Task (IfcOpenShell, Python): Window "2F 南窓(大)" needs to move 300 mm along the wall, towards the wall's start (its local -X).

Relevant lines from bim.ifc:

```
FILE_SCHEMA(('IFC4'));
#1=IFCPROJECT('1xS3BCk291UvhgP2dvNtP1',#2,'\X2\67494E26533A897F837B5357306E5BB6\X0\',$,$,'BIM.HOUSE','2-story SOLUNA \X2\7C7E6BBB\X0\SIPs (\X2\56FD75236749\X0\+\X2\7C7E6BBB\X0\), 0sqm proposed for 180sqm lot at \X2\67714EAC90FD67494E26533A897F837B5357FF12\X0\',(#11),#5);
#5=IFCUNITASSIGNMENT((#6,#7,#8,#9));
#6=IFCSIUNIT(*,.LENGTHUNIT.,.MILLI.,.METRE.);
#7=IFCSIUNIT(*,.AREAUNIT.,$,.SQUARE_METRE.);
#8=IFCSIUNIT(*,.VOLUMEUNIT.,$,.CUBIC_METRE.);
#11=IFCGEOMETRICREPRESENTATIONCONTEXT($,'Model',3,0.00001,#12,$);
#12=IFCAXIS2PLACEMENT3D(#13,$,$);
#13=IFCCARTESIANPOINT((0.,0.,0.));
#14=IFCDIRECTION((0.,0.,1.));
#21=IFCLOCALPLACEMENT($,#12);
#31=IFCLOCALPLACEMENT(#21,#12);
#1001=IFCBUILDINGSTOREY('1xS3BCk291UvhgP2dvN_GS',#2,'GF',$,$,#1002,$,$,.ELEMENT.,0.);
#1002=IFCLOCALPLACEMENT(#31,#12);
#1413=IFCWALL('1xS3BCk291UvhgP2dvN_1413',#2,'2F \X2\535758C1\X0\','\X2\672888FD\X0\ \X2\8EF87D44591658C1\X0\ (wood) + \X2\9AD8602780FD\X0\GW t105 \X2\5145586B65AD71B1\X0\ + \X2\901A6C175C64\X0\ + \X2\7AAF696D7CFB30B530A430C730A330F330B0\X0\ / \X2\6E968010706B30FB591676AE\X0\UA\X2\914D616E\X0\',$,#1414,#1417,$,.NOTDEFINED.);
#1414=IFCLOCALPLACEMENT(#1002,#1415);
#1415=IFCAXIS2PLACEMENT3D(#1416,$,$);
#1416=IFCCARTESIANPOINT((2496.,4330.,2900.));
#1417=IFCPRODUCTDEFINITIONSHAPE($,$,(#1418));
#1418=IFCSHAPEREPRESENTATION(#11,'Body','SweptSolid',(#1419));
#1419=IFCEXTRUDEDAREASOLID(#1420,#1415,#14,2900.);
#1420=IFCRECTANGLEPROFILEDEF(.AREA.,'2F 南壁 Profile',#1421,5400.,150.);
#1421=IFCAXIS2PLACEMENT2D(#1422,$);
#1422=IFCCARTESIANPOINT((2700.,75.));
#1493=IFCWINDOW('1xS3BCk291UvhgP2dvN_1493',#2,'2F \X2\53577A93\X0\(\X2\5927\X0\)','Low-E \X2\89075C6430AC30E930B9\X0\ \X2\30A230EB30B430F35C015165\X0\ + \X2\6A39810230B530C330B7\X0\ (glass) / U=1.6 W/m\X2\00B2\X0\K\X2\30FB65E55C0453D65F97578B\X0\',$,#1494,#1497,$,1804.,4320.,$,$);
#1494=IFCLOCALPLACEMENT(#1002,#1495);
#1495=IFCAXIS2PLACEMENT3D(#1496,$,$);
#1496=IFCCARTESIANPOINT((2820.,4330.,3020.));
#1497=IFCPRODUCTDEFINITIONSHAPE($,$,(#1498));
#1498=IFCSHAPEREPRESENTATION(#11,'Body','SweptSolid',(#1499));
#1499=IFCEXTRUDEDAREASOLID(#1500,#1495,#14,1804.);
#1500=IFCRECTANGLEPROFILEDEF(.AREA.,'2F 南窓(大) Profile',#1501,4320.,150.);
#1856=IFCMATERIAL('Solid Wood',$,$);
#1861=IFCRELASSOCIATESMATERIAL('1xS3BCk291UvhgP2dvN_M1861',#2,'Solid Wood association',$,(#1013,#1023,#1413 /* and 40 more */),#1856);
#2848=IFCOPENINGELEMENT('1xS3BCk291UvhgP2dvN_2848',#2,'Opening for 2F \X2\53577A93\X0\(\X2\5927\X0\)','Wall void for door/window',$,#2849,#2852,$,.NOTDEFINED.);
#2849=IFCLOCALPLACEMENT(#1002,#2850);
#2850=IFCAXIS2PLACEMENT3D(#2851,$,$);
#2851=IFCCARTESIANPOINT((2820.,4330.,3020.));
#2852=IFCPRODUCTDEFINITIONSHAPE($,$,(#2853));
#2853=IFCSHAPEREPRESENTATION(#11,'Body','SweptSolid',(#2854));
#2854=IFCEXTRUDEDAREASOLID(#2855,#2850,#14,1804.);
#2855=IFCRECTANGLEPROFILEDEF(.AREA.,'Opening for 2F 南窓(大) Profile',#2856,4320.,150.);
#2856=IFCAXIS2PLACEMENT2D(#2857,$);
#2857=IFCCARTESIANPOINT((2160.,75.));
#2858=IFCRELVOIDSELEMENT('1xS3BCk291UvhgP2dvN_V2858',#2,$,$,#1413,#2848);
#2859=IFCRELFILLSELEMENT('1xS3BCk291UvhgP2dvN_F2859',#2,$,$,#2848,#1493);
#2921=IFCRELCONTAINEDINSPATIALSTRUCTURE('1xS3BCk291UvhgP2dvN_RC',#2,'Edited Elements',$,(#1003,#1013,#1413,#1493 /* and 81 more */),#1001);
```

```python
import ifcopenshell
import ifcopenshell.api.geometry
import ifcopenshell.util.placement

model = ifcopenshell.open("bim.ifc")

window = model.by_guid("1xS3BCk291UvhgP2dvN_1493")
opening = window.FillsVoids[0].RelatingOpeningElement
wall = opening.VoidsElements[0].RelatingBuildingElement

wall_matrix = ifcopenshell.util.placement.get_local_placement(wall.ObjectPlacement)
shift = wall_matrix[:3, 0] * -300.0
before = ifcopenshell.util.placement.get_local_placement(window.ObjectPlacement)[:3, 3].copy()

# The window is not placed relative to its opening, so move both.
for product in (opening, window):
    matrix = ifcopenshell.util.placement.get_local_placement(product.ObjectPlacement)
    matrix[:3, 3] += shift
    ifcopenshell.api.geometry.edit_object_placement(model, product=product, matrix=matrix, is_si=False)

after = ifcopenshell.util.placement.get_local_placement(window.ObjectPlacement)[:3, 3]
print("window moved by", (after - before).round(3) + 0.0)

model.write("bim_updated.ifc")
```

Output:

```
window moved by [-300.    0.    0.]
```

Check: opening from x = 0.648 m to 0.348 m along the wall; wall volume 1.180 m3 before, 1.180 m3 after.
